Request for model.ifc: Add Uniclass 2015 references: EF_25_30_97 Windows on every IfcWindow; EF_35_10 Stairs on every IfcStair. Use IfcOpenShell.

First a look at what the model holds.

```python
import ifcopenshell

model = ifcopenshell.open("model.ifc")
print(model.schema)
print("classifications:", [c.Name for c in model.by_type("IfcClassification")])
for ifc_class in ("IfcDoor", "IfcRoof", "IfcStair", "IfcWall", "IfcWindow"):
    print(ifc_class, len(model.by_type(ifc_class)))
```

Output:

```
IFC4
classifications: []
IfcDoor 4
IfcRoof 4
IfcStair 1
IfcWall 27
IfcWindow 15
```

```python
import ifcopenshell
import ifcopenshell.api.classification

model = ifcopenshell.open("model.ifc")

system = ifcopenshell.api.classification.add_classification(model, classification="Uniclass 2015")

codes = {
    "IfcWindow": ("EF_25_30_97", "Windows"),
    "IfcStair": ("EF_35_10", "Stairs"),
}
for ifc_class, (code, name) in codes.items():
    products = model.by_type(ifc_class)
    ifcopenshell.api.classification.add_reference(
        model, products=products, classification=system, identification=code, name=name
    )
    print(code, len(products))

model.write("model_v2.ifc")
```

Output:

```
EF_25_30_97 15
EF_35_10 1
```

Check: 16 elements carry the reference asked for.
